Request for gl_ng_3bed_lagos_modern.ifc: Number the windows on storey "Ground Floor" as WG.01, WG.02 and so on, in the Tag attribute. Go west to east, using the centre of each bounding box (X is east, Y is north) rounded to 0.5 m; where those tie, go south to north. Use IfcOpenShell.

First a look at what the model holds.

```python
import ifcopenshell
import ifcopenshell.util.element
import ifcopenshell.util.placement

model = ifcopenshell.open("gl_ng_3bed_lagos_modern.ifc")
print(model.schema)
storey = next(s for s in model.by_type("IfcBuildingStorey") if s.Name == "Ground Floor")
windows = [e for e in ifcopenshell.util.element.get_decomposition(storey) if e.is_a("IfcWindow")]
for e in sorted(windows, key=lambda e: e.id()):
    origin = ifcopenshell.util.placement.get_local_placement(e.ObjectPlacement)[:3, 3]
    print(e.id(), e.Tag, e.Name, origin.round(2) + 0.0, sep=" | ")
```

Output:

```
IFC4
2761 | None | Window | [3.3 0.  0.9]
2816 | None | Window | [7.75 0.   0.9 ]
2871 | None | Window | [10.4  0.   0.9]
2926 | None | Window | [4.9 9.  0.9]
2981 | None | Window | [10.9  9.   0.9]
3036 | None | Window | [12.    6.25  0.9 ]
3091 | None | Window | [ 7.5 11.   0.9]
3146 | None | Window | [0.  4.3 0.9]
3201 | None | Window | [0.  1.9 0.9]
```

```python
import ifcopenshell
import ifcopenshell.geom
import ifcopenshell.util.element
import ifcopenshell.util.shape

model = ifcopenshell.open("gl_ng_3bed_lagos_modern.ifc")
settings = ifcopenshell.geom.settings()
settings.set("use-world-coords", True)


def centre(element):
    shape = ifcopenshell.geom.create_shape(settings, element)
    return ifcopenshell.util.shape.get_bbox_centroid(shape.geometry)


storey = next(s for s in model.by_type("IfcBuildingStorey") if s.Name == "Ground Floor")
windows = [e for e in ifcopenshell.util.element.get_decomposition(storey) if e.is_a("IfcWindow")]

# Insertion points can sit at a corner or the storey origin, so sort by the geometry (in metres).
centres = {e: centre(e) for e in windows}
windows.sort(key=lambda e: (round(centres[e][0] / 0.5), centres[e][1]))

for i, e in enumerate(windows, start=1):
    number = f"WG.{i:02d}"
    e.Tag = number
    print(e.id(), number)

model.write("gl_ng_3bed_lagos_modern_rev.ifc")
```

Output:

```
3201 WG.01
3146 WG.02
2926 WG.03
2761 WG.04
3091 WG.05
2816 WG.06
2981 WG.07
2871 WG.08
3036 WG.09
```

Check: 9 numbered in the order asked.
